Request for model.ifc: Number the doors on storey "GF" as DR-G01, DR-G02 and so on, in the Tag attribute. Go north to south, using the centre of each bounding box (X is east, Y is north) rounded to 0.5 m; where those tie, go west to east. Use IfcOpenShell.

First a look at what the model holds.

```python
import ifcopenshell
import ifcopenshell.util.element
import ifcopenshell.util.placement

model = ifcopenshell.open("model.ifc")
print(model.schema)
storey = next(s for s in model.by_type("IfcBuildingStorey") if s.Name == "GF")
doors = [e for e in ifcopenshell.util.element.get_decomposition(storey) if e.is_a("IfcDoor")]
for e in sorted(doors, key=lambda e: e.id()):
    origin = ifcopenshell.util.placement.get_local_placement(e.ObjectPlacement)[:3, 3]
    print(e.id(), e.Tag, e.Name, origin.round(2) + 0.0, sep=" | ")
```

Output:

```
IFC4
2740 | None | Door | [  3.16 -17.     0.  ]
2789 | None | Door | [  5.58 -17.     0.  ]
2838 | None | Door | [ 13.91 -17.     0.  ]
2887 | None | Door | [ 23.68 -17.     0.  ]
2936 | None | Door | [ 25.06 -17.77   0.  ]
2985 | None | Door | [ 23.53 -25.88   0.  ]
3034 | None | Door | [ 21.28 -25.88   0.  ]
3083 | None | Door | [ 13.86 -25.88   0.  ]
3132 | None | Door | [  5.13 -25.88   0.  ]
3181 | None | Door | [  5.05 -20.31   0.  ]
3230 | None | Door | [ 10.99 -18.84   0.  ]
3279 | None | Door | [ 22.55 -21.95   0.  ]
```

```python
import ifcopenshell
import ifcopenshell.geom
import ifcopenshell.util.element
import ifcopenshell.util.shape

model = ifcopenshell.open("model.ifc")
settings = ifcopenshell.geom.settings()
settings.set("use-world-coords", True)


def centre(element):
    shape = ifcopenshell.geom.create_shape(settings, element)
    return ifcopenshell.util.shape.get_bbox_centroid(shape.geometry)


storey = next(s for s in model.by_type("IfcBuildingStorey") if s.Name == "GF")
doors = [e for e in ifcopenshell.util.element.get_decomposition(storey) if e.is_a("IfcDoor")]

# Insertion points can sit at a corner or the storey origin, so sort by the geometry (in metres).
centres = {e: centre(e) for e in doors}
doors.sort(key=lambda e: (-round(centres[e][1] / 0.5), centres[e][0]))

for i, e in enumerate(doors, start=1):
    number = f"DR-G{i:02d}"
    e.Tag = number
    print(e.id(), number)

model.write("model_updated.ifc")
```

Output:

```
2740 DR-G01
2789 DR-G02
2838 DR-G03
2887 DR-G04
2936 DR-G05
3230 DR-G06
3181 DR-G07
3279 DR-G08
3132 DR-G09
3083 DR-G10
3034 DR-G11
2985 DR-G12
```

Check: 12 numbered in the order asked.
